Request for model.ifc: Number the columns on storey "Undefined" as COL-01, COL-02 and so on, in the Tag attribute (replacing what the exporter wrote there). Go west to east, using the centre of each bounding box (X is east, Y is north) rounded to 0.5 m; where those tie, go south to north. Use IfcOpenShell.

First a look at what the model holds.

```python
import ifcopenshell
import ifcopenshell.util.element
import ifcopenshell.util.placement

model = ifcopenshell.open("model.ifc")
print(model.schema)
storey = next(s for s in model.by_type("IfcBuildingStorey") if s.Name == "Undefined")
columns = [e for e in ifcopenshell.util.element.get_decomposition(storey) if e.is_a("IfcColumn")]
for e in sorted(columns, key=lambda e: e.id()):
    origin = ifcopenshell.util.placement.get_local_placement(e.ObjectPlacement)[:3, 3]
    print(e.id(), e.Tag, e.Name, origin.round(2) + 0.0, sep=" | ")
```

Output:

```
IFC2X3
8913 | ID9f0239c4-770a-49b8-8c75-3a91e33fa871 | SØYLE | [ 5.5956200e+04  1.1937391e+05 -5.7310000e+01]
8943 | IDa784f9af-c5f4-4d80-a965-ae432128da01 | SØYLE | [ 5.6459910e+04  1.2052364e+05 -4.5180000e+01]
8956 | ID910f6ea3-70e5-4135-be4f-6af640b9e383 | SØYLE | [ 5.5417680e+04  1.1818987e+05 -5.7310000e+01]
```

```python
import ifcopenshell
import ifcopenshell.geom
import ifcopenshell.util.element
import ifcopenshell.util.shape

model = ifcopenshell.open("model.ifc")
settings = ifcopenshell.geom.settings()
settings.set("use-world-coords", True)


def centre(element):
    shape = ifcopenshell.geom.create_shape(settings, element)
    return ifcopenshell.util.shape.get_bbox_centroid(shape.geometry)


storey = next(s for s in model.by_type("IfcBuildingStorey") if s.Name == "Undefined")
columns = [e for e in ifcopenshell.util.element.get_decomposition(storey) if e.is_a("IfcColumn")]

# Insertion points can sit at a corner or the storey origin, so sort by the geometry (in metres).
centres = {e: centre(e) for e in columns}
columns.sort(key=lambda e: (round(centres[e][0] / 0.5), centres[e][1]))

for i, e in enumerate(columns, start=1):
    number = f"COL-{i:02d}"
    e.Tag = number
    print(e.id(), number)

model.write("model_rev.ifc")
```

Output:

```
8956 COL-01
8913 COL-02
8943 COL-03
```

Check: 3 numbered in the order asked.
